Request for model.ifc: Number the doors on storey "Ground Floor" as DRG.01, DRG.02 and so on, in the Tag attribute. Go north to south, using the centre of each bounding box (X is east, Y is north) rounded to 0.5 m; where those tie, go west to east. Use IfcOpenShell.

First a look at what the model holds.

```python
import ifcopenshell
import ifcopenshell.util.element
import ifcopenshell.util.placement

model = ifcopenshell.open("model.ifc")
print(model.schema)
storey = next(s for s in model.by_type("IfcBuildingStorey") if s.Name == "Ground Floor")
doors = [e for e in ifcopenshell.util.element.get_decomposition(storey) if e.is_a("IfcDoor")]
for e in sorted(doors, key=lambda e: e.id()):
    origin = ifcopenshell.util.placement.get_local_placement(e.ObjectPlacement)[:3, 3]
    print(e.id(), e.Tag, e.Name, origin.round(2) + 0.0, sep=" | ")
```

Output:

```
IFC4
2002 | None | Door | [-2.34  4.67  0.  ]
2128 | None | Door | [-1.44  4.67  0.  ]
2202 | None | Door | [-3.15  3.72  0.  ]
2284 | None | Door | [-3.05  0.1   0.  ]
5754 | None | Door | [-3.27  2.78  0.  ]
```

```python
import ifcopenshell
import ifcopenshell.geom
import ifcopenshell.util.element
import ifcopenshell.util.shape

model = ifcopenshell.open("model.ifc")
settings = ifcopenshell.geom.settings()
settings.set("use-world-coords", True)


def centre(element):
    shape = ifcopenshell.geom.create_shape(settings, element)
    return ifcopenshell.util.shape.get_bbox_centroid(shape.geometry)


storey = next(s for s in model.by_type("IfcBuildingStorey") if s.Name == "Ground Floor")
doors = [e for e in ifcopenshell.util.element.get_decomposition(storey) if e.is_a("IfcDoor")]

# Insertion points can sit at a corner or the storey origin, so sort by the geometry (in metres).
centres = {e: centre(e) for e in doors}
doors.sort(key=lambda e: (-round(centres[e][1] / 0.5), centres[e][0]))

for i, e in enumerate(doors, start=1):
    number = f"DRG.{i:02d}"
    e.Tag = number
    print(e.id(), number)

model.write("model_edited.ifc")
```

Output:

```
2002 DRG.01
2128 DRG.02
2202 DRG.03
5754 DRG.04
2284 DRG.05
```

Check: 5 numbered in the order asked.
